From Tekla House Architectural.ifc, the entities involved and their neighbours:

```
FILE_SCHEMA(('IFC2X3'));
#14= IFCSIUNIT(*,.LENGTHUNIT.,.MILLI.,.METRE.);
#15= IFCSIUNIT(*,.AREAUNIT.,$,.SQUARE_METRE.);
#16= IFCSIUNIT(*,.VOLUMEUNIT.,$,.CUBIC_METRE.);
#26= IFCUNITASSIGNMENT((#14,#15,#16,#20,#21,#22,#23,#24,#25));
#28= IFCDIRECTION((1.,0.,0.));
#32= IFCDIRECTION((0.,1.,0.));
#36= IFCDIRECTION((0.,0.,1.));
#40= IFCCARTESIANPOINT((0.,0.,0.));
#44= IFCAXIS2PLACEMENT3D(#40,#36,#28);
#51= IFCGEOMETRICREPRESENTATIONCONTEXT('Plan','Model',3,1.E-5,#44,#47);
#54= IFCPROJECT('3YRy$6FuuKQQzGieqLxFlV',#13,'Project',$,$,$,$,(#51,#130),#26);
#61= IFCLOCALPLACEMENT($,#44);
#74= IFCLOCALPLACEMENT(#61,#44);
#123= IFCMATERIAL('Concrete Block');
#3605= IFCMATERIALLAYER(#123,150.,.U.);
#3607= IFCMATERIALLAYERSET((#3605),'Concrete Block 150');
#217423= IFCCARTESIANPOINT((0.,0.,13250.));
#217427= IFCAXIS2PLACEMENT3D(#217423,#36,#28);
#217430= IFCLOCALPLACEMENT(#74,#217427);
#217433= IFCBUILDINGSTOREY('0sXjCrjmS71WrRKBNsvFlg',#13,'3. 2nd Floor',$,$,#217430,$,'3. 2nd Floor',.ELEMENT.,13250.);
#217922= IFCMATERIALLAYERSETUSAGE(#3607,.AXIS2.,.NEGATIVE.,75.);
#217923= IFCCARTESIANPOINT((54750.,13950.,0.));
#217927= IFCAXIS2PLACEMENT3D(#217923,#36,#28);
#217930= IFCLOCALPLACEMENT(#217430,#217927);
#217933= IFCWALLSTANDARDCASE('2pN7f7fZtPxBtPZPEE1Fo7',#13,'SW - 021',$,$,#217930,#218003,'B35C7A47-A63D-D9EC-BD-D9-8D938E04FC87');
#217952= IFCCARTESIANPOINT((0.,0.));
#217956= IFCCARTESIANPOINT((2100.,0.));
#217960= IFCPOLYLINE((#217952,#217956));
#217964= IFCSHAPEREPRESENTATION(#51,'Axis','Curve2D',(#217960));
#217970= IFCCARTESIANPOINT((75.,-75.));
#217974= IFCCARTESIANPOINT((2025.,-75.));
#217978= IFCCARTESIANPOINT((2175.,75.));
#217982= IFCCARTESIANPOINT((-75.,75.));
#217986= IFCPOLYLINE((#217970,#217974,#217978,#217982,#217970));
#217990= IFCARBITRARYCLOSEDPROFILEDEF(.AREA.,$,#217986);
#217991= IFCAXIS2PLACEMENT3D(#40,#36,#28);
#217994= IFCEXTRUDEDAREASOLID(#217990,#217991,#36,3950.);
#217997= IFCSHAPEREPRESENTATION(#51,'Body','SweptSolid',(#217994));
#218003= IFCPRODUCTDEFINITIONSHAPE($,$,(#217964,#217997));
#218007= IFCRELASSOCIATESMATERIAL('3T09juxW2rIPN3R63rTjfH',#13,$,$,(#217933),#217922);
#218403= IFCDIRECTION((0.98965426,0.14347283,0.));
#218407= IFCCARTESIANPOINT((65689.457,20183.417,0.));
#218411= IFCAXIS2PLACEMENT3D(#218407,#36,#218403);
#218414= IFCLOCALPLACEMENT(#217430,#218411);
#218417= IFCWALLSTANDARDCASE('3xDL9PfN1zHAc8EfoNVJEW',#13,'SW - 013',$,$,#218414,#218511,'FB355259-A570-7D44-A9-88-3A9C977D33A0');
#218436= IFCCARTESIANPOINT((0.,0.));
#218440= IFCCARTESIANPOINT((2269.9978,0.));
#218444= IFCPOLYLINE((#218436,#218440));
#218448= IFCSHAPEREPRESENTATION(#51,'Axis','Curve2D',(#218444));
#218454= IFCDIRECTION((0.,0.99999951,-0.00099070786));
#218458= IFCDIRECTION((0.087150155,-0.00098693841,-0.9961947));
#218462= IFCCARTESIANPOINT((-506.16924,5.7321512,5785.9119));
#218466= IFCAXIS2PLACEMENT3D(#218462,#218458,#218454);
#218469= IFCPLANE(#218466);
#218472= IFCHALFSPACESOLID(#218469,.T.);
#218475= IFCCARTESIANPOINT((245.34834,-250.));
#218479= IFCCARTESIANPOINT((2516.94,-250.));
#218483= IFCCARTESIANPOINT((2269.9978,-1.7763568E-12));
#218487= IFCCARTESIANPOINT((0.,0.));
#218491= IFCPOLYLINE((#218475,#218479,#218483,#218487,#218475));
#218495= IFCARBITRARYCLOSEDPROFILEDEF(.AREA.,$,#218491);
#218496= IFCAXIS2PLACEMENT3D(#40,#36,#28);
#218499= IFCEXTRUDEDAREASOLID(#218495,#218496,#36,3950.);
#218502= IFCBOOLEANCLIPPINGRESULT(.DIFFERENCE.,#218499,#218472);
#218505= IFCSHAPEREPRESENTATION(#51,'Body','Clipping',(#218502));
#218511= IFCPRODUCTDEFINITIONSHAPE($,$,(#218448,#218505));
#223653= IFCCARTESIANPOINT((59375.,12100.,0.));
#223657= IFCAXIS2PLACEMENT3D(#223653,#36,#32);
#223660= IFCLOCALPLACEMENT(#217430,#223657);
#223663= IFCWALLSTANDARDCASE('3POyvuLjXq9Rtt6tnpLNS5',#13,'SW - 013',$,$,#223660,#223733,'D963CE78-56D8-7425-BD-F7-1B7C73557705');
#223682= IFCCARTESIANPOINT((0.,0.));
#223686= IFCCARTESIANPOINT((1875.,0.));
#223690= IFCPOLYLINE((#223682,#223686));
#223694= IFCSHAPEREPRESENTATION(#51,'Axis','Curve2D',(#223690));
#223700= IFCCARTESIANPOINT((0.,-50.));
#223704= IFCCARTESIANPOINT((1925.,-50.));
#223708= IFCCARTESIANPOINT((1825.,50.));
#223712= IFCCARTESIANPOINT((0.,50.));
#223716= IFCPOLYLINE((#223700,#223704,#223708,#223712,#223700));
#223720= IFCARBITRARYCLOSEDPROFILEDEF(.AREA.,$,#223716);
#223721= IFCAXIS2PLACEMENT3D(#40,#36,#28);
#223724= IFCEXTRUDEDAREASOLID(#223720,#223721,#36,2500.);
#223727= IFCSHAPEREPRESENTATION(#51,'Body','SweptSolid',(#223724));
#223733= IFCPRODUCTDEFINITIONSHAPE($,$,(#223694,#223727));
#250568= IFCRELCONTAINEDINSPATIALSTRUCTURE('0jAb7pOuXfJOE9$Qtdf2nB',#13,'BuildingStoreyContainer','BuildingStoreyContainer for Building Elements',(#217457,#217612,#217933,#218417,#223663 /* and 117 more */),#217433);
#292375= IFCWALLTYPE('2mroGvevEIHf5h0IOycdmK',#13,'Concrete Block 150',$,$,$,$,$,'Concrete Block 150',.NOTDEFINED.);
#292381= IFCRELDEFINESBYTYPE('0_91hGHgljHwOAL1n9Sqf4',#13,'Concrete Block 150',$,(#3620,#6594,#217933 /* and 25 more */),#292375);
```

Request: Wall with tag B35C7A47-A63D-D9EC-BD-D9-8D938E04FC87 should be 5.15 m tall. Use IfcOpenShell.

```python
import ifcopenshell
import ifcopenshell.geom
import ifcopenshell.util.shape
import ifcopenshell.util.unit

model = ifcopenshell.open("Tekla House Architectural.ifc")
unit_scale = ifcopenshell.util.unit.calculate_unit_scale(model)
settings = ifcopenshell.geom.settings()


def volume(element):
    """Net volume in cubic metres, openings subtracted."""
    shape = ifcopenshell.geom.create_shape(settings, element)
    return ifcopenshell.util.shape.get_volume(shape.geometry)


wall = model.by_id(217933)
before = volume(wall)

body = next(r for r in wall.Representation.Representations if r.RepresentationIdentifier == "Body")
solid = body.Items[0]
old_height = solid.Depth
solid.Depth = 5.15 / unit_scale
after = volume(wall)

print(f"height {old_height:g} -> {solid.Depth:g}, volume {before:.3f} -> {after:.3f} m3")

model.write("Tekla House Architectural_edited.ifc")
```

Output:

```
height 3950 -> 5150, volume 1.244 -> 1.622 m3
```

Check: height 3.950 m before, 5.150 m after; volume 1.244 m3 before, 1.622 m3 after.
